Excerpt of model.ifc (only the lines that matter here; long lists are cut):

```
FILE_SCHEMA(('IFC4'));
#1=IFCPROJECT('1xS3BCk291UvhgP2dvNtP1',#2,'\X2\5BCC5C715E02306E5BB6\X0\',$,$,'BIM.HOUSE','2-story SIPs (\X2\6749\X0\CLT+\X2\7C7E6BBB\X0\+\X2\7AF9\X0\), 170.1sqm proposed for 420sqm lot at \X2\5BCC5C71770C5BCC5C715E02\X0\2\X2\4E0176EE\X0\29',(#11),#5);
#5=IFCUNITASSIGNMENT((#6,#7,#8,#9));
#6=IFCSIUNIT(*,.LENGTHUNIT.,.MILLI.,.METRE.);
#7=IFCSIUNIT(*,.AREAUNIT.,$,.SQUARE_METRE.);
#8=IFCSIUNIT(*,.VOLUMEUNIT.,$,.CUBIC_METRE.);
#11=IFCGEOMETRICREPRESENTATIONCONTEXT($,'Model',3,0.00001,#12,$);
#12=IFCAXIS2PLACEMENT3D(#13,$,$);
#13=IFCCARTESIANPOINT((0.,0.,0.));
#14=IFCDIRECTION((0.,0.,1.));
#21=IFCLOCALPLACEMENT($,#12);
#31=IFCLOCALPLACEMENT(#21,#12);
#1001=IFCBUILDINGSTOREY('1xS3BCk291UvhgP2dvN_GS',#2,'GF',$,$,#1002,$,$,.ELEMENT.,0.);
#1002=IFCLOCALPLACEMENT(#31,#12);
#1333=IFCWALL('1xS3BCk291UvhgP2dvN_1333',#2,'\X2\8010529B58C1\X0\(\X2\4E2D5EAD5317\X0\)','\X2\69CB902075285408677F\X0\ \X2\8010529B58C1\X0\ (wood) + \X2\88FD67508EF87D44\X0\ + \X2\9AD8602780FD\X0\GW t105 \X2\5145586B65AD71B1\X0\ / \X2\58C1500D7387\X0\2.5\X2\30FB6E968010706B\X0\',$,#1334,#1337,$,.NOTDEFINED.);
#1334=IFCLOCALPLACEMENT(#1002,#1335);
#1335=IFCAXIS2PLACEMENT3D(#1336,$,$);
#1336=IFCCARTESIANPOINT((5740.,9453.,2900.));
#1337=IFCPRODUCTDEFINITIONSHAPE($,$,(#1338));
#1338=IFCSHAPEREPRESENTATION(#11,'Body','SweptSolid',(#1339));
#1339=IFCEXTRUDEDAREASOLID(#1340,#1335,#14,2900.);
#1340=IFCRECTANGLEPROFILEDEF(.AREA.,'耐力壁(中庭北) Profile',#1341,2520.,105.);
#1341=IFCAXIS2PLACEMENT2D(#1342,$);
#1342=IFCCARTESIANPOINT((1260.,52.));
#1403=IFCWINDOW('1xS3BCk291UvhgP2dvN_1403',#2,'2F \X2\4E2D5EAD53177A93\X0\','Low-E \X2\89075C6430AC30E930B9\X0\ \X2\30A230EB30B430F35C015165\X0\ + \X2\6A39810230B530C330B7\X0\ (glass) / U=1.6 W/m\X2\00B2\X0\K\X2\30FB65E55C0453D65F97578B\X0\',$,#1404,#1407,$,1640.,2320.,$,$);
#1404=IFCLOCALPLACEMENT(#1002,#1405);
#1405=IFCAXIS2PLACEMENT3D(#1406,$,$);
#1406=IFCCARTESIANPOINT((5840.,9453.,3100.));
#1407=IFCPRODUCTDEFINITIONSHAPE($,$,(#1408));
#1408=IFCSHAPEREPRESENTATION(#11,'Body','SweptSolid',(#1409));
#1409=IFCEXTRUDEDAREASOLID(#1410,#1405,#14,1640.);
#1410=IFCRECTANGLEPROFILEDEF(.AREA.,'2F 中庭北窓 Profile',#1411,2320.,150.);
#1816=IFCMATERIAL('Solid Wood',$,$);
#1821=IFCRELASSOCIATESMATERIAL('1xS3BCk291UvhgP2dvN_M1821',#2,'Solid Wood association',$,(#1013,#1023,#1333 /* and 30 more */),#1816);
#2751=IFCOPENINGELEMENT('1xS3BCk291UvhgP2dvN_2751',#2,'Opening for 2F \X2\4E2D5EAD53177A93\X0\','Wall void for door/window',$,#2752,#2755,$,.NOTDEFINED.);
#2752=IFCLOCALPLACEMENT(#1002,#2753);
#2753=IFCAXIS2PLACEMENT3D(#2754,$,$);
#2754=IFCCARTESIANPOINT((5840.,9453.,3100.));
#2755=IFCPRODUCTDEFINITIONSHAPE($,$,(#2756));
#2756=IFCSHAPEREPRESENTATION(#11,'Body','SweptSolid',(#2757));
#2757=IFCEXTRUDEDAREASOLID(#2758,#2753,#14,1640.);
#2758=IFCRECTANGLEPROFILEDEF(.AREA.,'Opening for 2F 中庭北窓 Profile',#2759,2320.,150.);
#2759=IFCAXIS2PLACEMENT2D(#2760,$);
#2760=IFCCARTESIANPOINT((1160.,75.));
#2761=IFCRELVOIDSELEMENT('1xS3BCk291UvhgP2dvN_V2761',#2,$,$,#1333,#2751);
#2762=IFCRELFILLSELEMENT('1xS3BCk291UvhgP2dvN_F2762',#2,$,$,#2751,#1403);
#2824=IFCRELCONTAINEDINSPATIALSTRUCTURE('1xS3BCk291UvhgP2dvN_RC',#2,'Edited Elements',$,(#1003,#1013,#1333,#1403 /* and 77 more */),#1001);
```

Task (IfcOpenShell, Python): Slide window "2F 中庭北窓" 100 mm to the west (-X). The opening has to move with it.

```python
import ifcopenshell
import ifcopenshell.api.geometry
import ifcopenshell.util.placement

model = ifcopenshell.open("model.ifc")

window = model.by_guid("1xS3BCk291UvhgP2dvN_1403")
opening = window.FillsVoids[0].RelatingOpeningElement
wall = opening.VoidsElements[0].RelatingBuildingElement

wall_matrix = ifcopenshell.util.placement.get_local_placement(wall.ObjectPlacement)
shift = wall_matrix[:3, 0] * -100.0
before = ifcopenshell.util.placement.get_local_placement(window.ObjectPlacement)[:3, 3].copy()

# The window is not placed relative to its opening, so move both.
for product in (opening, window):
    matrix = ifcopenshell.util.placement.get_local_placement(product.ObjectPlacement)
    matrix[:3, 3] += shift
    ifcopenshell.api.geometry.edit_object_placement(model, product=product, matrix=matrix, is_si=False)

after = ifcopenshell.util.placement.get_local_placement(window.ObjectPlacement)[:3, 3]
print("window moved by", (after - before).round(3) + 0.0)

model.write("model_edited.ifc")
```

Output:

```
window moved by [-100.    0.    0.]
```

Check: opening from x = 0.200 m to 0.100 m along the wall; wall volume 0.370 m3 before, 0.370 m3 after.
